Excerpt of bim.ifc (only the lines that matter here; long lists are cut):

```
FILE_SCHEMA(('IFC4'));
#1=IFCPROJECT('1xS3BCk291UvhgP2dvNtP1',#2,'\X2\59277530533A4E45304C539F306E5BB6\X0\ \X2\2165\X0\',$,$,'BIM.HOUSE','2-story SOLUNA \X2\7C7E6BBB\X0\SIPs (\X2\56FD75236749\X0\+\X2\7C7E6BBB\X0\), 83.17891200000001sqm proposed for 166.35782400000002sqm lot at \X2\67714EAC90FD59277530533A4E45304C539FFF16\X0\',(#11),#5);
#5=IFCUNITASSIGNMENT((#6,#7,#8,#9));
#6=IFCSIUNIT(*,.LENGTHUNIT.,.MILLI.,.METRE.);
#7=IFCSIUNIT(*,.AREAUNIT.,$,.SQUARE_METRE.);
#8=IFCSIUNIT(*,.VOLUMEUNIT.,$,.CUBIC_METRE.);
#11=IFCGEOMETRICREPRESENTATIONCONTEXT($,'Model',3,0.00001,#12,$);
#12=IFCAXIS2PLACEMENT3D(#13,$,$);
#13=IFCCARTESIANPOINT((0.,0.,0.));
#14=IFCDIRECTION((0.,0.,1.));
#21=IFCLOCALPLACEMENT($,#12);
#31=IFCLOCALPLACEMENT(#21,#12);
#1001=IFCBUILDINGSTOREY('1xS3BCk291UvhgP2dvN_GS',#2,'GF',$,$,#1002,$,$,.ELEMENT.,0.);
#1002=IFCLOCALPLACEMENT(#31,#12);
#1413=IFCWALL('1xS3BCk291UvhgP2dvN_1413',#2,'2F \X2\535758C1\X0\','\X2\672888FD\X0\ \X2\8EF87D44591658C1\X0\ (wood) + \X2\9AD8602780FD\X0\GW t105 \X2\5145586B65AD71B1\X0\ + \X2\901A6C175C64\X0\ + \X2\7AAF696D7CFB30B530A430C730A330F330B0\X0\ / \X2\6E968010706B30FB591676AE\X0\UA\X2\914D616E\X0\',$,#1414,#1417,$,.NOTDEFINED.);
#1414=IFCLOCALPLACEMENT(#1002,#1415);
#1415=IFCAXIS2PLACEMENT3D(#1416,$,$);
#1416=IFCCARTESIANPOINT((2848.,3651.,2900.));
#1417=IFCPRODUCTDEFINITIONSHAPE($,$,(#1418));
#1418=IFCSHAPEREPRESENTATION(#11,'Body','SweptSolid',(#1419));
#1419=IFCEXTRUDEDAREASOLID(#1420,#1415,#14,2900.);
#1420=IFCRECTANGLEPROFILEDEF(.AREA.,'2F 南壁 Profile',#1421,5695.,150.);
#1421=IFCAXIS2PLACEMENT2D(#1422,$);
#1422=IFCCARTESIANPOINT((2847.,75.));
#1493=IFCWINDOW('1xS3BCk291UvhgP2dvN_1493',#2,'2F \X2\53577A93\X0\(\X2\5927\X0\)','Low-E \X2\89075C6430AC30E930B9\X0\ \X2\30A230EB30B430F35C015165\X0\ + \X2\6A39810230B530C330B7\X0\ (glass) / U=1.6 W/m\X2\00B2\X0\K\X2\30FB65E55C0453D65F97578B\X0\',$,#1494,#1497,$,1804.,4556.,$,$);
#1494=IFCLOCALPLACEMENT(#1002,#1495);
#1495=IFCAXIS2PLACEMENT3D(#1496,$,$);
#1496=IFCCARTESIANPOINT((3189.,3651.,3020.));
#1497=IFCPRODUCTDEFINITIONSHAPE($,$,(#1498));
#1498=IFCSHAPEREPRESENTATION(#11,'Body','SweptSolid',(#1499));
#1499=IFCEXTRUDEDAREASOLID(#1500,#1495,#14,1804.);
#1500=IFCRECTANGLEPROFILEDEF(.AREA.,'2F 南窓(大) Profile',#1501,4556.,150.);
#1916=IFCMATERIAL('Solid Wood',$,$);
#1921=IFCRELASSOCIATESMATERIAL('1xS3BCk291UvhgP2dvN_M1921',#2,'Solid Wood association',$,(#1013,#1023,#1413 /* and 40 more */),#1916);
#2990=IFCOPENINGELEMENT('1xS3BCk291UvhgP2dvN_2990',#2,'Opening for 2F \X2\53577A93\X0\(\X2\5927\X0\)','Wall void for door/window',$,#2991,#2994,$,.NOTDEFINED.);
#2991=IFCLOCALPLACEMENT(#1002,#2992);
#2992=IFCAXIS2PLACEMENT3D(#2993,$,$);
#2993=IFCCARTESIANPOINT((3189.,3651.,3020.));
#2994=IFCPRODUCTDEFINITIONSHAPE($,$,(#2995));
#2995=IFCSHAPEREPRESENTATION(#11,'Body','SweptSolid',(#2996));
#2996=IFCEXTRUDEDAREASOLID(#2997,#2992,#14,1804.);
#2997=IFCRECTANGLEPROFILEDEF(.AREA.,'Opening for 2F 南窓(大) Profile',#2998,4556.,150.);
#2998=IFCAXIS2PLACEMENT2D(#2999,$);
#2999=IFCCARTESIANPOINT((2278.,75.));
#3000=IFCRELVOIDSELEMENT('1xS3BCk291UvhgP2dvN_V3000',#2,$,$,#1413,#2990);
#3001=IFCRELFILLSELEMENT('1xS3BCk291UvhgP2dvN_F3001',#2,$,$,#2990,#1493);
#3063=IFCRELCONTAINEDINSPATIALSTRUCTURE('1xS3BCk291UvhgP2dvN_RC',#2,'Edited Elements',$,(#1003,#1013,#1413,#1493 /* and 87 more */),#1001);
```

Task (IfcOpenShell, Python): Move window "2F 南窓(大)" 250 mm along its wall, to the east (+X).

```python
import ifcopenshell
import ifcopenshell.api.geometry
import ifcopenshell.util.placement

model = ifcopenshell.open("bim.ifc")

window = model.by_guid("1xS3BCk291UvhgP2dvN_1493")
opening = window.FillsVoids[0].RelatingOpeningElement
wall = opening.VoidsElements[0].RelatingBuildingElement

wall_matrix = ifcopenshell.util.placement.get_local_placement(wall.ObjectPlacement)
shift = wall_matrix[:3, 0] * 250.0
before = ifcopenshell.util.placement.get_local_placement(window.ObjectPlacement)[:3, 3].copy()

# The window is not placed relative to its opening, so move both.
for product in (opening, window):
    matrix = ifcopenshell.util.placement.get_local_placement(product.ObjectPlacement)
    matrix[:3, 3] += shift
    ifcopenshell.api.geometry.edit_object_placement(model, product=product, matrix=matrix, is_si=False)

after = ifcopenshell.util.placement.get_local_placement(window.ObjectPlacement)[:3, 3]
print("window moved by", (after - before).round(3) + 0.0)

model.write("bim_v2.ifc")
```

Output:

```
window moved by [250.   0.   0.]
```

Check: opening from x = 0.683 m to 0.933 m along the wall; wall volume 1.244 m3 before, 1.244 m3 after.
